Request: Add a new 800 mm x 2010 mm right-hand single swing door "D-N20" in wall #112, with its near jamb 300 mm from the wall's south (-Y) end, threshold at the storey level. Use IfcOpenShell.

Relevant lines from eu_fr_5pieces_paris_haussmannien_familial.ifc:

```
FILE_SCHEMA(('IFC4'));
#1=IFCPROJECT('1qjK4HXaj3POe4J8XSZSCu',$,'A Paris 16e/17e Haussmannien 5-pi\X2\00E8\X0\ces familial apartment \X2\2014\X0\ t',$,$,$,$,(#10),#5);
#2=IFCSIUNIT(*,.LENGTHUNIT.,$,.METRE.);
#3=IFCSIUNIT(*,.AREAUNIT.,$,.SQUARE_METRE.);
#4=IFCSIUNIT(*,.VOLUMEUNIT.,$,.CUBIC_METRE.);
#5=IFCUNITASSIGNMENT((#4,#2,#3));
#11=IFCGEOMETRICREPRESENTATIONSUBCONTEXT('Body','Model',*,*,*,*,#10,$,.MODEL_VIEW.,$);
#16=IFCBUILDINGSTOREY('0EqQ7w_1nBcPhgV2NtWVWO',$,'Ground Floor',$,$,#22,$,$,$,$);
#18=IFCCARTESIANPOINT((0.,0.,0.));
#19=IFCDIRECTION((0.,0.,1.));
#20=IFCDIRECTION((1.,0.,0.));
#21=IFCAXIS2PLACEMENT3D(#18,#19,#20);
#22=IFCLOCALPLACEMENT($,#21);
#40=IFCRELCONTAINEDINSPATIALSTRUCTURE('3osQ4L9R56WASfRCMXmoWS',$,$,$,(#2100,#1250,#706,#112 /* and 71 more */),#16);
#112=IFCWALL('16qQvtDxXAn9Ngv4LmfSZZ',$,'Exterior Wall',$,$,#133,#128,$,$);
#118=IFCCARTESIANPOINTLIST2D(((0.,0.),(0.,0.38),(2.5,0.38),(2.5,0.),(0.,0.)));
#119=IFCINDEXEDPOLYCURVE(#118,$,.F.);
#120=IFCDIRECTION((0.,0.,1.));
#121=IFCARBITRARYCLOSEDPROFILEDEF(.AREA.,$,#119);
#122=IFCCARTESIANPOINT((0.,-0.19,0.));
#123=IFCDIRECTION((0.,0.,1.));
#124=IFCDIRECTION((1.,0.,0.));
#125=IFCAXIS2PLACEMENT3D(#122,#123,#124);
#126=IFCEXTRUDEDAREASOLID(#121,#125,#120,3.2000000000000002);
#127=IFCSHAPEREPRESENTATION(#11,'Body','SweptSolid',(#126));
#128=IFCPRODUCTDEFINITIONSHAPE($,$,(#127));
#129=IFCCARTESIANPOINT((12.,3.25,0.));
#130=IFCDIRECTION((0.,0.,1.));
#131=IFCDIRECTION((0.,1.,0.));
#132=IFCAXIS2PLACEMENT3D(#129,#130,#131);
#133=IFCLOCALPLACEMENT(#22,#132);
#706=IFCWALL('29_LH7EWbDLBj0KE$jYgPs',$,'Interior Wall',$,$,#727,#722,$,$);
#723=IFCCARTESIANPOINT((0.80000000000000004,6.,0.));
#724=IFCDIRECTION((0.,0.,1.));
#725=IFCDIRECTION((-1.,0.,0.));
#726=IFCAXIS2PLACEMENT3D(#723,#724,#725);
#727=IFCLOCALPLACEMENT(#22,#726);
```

```python
import numpy as np
import ifcopenshell
import ifcopenshell.api.feature
import ifcopenshell.api.geometry
import ifcopenshell.api.root
import ifcopenshell.api.spatial
import ifcopenshell.geom
import ifcopenshell.util.element
import ifcopenshell.util.placement
import ifcopenshell.util.representation
import ifcopenshell.util.shape
import ifcopenshell.util.unit

model = ifcopenshell.open("eu_fr_5pieces_paris_haussmannien_familial.ifc")
unit_scale = ifcopenshell.util.unit.calculate_unit_scale(model)
settings = ifcopenshell.geom.settings()


def volume(element):
    """Net volume in cubic metres, openings subtracted."""
    shape = ifcopenshell.geom.create_shape(settings, element)
    return ifcopenshell.util.shape.get_volume(shape.geometry)


wall = model.by_guid("16qQvtDxXAn9Ngv4LmfSZZ")
storey = ifcopenshell.util.element.get_container(wall, ifc_class="IfcBuildingStorey")
context = ifcopenshell.util.representation.get_context(model, "Model", "Body", "MODEL_VIEW")
before = volume(wall)

width, height, from_end, sill = 0.8, 2.01, 0.3, 0.0  # metres

# The wall runs along its own X axis, and the end named is its -X end.
wall_shape = ifcopenshell.geom.create_shape(settings, wall)
x, y, z = ifcopenshell.util.shape.get_vertices(wall_shape.geometry).T
start = x.min() + from_end
face, thickness = float(y.min()), float(y.max() - y.min())
wall_matrix = ifcopenshell.util.placement.get_local_placement(wall.ObjectPlacement)
level = ifcopenshell.util.placement.get_local_placement(storey.ObjectPlacement)[2, 3]


def in_wall(x, y):
    """Placement at x, y metres in the wall's axes, at sill height."""
    matrix = wall_matrix.copy()
    matrix[:, 3] = wall_matrix @ np.array([x / unit_scale, y / unit_scale, 0.0, 1.0])
    matrix[2, 3] = level + sill / unit_scale
    return matrix


# Opening: a box that overshoots both wall faces by 50 mm.
opening = ifcopenshell.api.root.create_entity(model, ifc_class="IfcOpeningElement", predefined_type="OPENING")
box = ifcopenshell.api.geometry.add_wall_representation(
    model, context=context, length=width, height=height, thickness=thickness + 0.1
)
ifcopenshell.api.geometry.assign_representation(model, product=opening, representation=box)
ifcopenshell.api.geometry.edit_object_placement(model, product=opening, matrix=in_wall(start, face - 0.05), is_si=False)
ifcopenshell.api.feature.add_feature(model, feature=opening, element=wall)

door = ifcopenshell.api.root.create_entity(model, ifc_class="IfcDoor", name="D-N20", predefined_type="DOOR")
door.OverallWidth, door.OverallHeight = width / unit_scale, height / unit_scale
door.OperationType = "SINGLE_SWING_RIGHT"
body = ifcopenshell.api.geometry.add_door_representation(
    model,
    context=context,
    overall_width=door.OverallWidth,
    overall_height=door.OverallHeight,
    operation_type="SINGLE_SWING_RIGHT",
    lining_properties={"LiningDepth": thickness / unit_scale, "ThresholdDepth": thickness / unit_scale},
)
ifcopenshell.api.geometry.assign_representation(model, product=door, representation=body)
ifcopenshell.api.spatial.assign_container(model, products=[door], relating_structure=storey)
ifcopenshell.api.feature.add_filling(model, opening=opening, element=door)

# The lining spans the wall, so the door starts at the wall face.
ifcopenshell.api.geometry.edit_object_placement(model, product=door, matrix=in_wall(start, face), is_si=False)

after = volume(wall)

print(f"wall volume {before:.3f} -> {after:.3f} m3")

model.write("eu_fr_5pieces_paris_haussmannien_familial_v2.ifc")
```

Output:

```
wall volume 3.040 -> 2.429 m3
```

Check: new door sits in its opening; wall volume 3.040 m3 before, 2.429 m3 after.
